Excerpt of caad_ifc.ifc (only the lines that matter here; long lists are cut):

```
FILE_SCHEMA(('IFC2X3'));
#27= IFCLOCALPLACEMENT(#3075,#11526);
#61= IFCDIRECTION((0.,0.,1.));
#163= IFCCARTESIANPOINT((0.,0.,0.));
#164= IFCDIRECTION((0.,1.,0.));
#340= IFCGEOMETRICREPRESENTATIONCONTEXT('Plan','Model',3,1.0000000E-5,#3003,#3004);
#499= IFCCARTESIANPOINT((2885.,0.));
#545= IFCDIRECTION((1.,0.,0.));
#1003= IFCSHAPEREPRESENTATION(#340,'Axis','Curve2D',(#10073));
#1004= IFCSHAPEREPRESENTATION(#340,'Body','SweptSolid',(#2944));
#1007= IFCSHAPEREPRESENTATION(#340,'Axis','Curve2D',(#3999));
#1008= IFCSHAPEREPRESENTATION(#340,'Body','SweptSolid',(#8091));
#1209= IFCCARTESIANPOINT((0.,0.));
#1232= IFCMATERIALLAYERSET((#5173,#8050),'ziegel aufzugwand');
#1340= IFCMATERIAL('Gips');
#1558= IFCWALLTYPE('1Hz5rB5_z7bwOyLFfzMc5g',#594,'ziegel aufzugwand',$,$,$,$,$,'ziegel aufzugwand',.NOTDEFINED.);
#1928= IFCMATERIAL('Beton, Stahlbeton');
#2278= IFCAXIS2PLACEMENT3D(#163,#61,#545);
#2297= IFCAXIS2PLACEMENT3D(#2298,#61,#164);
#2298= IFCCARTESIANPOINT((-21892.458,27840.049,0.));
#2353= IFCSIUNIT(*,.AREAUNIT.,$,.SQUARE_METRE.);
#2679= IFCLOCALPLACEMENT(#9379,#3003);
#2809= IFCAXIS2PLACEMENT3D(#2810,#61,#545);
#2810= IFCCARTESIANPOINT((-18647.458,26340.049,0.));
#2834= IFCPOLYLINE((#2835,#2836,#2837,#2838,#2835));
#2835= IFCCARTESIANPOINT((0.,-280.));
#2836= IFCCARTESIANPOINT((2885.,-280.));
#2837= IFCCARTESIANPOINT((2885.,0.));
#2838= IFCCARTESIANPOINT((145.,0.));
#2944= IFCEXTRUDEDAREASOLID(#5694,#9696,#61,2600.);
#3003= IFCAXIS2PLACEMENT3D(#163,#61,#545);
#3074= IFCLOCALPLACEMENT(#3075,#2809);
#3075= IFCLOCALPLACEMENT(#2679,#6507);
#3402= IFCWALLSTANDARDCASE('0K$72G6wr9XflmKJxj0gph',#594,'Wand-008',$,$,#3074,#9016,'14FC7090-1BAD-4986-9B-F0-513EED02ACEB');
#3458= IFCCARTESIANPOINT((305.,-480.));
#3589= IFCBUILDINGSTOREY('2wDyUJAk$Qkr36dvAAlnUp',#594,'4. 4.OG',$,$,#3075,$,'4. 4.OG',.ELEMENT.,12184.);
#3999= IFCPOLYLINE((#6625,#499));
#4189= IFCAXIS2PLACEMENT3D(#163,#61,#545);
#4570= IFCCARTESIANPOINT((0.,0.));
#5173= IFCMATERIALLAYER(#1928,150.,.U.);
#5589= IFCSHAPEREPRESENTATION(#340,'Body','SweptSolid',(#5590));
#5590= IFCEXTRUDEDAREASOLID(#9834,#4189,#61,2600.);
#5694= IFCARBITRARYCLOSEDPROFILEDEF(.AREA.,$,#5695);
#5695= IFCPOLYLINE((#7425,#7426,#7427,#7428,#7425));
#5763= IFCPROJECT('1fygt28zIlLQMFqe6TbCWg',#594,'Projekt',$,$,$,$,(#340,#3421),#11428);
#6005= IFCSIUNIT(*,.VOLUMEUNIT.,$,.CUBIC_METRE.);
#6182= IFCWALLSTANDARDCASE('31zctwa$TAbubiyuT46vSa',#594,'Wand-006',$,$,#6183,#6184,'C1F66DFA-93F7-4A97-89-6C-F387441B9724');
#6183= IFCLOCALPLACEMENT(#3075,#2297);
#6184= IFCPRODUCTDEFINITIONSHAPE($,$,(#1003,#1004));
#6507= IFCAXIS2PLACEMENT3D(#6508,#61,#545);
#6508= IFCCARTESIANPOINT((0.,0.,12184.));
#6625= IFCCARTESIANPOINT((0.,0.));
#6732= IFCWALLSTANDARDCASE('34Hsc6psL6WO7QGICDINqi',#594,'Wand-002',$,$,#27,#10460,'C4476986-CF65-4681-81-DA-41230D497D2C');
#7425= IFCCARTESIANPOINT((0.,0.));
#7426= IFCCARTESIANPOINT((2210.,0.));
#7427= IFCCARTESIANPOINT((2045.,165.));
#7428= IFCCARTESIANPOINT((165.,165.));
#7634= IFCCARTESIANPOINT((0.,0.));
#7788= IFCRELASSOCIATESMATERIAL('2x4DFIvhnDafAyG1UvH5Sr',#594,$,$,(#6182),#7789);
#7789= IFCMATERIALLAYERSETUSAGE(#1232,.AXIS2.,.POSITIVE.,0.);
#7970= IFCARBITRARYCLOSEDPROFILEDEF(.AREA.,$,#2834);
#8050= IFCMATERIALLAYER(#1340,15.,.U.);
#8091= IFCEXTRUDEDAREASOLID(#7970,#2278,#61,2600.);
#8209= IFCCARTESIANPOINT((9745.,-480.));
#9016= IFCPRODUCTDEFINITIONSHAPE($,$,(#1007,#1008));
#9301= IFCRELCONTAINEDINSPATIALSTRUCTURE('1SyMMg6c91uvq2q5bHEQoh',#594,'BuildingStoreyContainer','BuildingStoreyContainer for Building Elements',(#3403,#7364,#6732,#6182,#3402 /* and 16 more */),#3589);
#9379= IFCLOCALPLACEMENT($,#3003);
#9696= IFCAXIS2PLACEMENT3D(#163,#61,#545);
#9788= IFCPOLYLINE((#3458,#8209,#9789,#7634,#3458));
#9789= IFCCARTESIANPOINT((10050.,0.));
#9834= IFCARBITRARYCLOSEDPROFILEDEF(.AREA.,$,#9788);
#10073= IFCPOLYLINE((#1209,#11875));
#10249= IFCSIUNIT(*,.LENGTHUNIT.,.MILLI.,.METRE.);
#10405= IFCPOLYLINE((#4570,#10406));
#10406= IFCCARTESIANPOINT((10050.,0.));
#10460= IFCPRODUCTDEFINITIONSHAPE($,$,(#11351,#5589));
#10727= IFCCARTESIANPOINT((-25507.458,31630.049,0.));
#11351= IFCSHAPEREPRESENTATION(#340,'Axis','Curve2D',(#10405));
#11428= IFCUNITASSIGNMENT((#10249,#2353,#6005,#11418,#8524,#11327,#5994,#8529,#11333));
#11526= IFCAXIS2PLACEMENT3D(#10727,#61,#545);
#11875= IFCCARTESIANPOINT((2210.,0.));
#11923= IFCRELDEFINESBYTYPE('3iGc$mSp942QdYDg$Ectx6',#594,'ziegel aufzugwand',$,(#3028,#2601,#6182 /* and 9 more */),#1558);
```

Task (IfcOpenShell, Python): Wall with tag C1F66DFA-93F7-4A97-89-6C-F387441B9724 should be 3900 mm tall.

```python
import ifcopenshell
import ifcopenshell.geom
import ifcopenshell.util.shape

model = ifcopenshell.open("caad_ifc.ifc")
settings = ifcopenshell.geom.settings()


def volume(element):
    """Net volume in cubic metres, openings subtracted."""
    shape = ifcopenshell.geom.create_shape(settings, element)
    return ifcopenshell.util.shape.get_volume(shape.geometry)


wall = model.by_guid("31zctwa$TAbubiyuT46vSa")
before = volume(wall)

body = next(r for r in wall.Representation.Representations if r.RepresentationIdentifier == "Body")
solid = body.Items[0]
old_height = solid.Depth
solid.Depth = 3900.0
after = volume(wall)

print(f"height {old_height:g} -> {solid.Depth:g}, volume {before:.3f} -> {after:.3f} m3")

model.write("caad_ifc_v2.ifc")
```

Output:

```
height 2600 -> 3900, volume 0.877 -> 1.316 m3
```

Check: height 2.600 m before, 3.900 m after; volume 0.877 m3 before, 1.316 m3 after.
